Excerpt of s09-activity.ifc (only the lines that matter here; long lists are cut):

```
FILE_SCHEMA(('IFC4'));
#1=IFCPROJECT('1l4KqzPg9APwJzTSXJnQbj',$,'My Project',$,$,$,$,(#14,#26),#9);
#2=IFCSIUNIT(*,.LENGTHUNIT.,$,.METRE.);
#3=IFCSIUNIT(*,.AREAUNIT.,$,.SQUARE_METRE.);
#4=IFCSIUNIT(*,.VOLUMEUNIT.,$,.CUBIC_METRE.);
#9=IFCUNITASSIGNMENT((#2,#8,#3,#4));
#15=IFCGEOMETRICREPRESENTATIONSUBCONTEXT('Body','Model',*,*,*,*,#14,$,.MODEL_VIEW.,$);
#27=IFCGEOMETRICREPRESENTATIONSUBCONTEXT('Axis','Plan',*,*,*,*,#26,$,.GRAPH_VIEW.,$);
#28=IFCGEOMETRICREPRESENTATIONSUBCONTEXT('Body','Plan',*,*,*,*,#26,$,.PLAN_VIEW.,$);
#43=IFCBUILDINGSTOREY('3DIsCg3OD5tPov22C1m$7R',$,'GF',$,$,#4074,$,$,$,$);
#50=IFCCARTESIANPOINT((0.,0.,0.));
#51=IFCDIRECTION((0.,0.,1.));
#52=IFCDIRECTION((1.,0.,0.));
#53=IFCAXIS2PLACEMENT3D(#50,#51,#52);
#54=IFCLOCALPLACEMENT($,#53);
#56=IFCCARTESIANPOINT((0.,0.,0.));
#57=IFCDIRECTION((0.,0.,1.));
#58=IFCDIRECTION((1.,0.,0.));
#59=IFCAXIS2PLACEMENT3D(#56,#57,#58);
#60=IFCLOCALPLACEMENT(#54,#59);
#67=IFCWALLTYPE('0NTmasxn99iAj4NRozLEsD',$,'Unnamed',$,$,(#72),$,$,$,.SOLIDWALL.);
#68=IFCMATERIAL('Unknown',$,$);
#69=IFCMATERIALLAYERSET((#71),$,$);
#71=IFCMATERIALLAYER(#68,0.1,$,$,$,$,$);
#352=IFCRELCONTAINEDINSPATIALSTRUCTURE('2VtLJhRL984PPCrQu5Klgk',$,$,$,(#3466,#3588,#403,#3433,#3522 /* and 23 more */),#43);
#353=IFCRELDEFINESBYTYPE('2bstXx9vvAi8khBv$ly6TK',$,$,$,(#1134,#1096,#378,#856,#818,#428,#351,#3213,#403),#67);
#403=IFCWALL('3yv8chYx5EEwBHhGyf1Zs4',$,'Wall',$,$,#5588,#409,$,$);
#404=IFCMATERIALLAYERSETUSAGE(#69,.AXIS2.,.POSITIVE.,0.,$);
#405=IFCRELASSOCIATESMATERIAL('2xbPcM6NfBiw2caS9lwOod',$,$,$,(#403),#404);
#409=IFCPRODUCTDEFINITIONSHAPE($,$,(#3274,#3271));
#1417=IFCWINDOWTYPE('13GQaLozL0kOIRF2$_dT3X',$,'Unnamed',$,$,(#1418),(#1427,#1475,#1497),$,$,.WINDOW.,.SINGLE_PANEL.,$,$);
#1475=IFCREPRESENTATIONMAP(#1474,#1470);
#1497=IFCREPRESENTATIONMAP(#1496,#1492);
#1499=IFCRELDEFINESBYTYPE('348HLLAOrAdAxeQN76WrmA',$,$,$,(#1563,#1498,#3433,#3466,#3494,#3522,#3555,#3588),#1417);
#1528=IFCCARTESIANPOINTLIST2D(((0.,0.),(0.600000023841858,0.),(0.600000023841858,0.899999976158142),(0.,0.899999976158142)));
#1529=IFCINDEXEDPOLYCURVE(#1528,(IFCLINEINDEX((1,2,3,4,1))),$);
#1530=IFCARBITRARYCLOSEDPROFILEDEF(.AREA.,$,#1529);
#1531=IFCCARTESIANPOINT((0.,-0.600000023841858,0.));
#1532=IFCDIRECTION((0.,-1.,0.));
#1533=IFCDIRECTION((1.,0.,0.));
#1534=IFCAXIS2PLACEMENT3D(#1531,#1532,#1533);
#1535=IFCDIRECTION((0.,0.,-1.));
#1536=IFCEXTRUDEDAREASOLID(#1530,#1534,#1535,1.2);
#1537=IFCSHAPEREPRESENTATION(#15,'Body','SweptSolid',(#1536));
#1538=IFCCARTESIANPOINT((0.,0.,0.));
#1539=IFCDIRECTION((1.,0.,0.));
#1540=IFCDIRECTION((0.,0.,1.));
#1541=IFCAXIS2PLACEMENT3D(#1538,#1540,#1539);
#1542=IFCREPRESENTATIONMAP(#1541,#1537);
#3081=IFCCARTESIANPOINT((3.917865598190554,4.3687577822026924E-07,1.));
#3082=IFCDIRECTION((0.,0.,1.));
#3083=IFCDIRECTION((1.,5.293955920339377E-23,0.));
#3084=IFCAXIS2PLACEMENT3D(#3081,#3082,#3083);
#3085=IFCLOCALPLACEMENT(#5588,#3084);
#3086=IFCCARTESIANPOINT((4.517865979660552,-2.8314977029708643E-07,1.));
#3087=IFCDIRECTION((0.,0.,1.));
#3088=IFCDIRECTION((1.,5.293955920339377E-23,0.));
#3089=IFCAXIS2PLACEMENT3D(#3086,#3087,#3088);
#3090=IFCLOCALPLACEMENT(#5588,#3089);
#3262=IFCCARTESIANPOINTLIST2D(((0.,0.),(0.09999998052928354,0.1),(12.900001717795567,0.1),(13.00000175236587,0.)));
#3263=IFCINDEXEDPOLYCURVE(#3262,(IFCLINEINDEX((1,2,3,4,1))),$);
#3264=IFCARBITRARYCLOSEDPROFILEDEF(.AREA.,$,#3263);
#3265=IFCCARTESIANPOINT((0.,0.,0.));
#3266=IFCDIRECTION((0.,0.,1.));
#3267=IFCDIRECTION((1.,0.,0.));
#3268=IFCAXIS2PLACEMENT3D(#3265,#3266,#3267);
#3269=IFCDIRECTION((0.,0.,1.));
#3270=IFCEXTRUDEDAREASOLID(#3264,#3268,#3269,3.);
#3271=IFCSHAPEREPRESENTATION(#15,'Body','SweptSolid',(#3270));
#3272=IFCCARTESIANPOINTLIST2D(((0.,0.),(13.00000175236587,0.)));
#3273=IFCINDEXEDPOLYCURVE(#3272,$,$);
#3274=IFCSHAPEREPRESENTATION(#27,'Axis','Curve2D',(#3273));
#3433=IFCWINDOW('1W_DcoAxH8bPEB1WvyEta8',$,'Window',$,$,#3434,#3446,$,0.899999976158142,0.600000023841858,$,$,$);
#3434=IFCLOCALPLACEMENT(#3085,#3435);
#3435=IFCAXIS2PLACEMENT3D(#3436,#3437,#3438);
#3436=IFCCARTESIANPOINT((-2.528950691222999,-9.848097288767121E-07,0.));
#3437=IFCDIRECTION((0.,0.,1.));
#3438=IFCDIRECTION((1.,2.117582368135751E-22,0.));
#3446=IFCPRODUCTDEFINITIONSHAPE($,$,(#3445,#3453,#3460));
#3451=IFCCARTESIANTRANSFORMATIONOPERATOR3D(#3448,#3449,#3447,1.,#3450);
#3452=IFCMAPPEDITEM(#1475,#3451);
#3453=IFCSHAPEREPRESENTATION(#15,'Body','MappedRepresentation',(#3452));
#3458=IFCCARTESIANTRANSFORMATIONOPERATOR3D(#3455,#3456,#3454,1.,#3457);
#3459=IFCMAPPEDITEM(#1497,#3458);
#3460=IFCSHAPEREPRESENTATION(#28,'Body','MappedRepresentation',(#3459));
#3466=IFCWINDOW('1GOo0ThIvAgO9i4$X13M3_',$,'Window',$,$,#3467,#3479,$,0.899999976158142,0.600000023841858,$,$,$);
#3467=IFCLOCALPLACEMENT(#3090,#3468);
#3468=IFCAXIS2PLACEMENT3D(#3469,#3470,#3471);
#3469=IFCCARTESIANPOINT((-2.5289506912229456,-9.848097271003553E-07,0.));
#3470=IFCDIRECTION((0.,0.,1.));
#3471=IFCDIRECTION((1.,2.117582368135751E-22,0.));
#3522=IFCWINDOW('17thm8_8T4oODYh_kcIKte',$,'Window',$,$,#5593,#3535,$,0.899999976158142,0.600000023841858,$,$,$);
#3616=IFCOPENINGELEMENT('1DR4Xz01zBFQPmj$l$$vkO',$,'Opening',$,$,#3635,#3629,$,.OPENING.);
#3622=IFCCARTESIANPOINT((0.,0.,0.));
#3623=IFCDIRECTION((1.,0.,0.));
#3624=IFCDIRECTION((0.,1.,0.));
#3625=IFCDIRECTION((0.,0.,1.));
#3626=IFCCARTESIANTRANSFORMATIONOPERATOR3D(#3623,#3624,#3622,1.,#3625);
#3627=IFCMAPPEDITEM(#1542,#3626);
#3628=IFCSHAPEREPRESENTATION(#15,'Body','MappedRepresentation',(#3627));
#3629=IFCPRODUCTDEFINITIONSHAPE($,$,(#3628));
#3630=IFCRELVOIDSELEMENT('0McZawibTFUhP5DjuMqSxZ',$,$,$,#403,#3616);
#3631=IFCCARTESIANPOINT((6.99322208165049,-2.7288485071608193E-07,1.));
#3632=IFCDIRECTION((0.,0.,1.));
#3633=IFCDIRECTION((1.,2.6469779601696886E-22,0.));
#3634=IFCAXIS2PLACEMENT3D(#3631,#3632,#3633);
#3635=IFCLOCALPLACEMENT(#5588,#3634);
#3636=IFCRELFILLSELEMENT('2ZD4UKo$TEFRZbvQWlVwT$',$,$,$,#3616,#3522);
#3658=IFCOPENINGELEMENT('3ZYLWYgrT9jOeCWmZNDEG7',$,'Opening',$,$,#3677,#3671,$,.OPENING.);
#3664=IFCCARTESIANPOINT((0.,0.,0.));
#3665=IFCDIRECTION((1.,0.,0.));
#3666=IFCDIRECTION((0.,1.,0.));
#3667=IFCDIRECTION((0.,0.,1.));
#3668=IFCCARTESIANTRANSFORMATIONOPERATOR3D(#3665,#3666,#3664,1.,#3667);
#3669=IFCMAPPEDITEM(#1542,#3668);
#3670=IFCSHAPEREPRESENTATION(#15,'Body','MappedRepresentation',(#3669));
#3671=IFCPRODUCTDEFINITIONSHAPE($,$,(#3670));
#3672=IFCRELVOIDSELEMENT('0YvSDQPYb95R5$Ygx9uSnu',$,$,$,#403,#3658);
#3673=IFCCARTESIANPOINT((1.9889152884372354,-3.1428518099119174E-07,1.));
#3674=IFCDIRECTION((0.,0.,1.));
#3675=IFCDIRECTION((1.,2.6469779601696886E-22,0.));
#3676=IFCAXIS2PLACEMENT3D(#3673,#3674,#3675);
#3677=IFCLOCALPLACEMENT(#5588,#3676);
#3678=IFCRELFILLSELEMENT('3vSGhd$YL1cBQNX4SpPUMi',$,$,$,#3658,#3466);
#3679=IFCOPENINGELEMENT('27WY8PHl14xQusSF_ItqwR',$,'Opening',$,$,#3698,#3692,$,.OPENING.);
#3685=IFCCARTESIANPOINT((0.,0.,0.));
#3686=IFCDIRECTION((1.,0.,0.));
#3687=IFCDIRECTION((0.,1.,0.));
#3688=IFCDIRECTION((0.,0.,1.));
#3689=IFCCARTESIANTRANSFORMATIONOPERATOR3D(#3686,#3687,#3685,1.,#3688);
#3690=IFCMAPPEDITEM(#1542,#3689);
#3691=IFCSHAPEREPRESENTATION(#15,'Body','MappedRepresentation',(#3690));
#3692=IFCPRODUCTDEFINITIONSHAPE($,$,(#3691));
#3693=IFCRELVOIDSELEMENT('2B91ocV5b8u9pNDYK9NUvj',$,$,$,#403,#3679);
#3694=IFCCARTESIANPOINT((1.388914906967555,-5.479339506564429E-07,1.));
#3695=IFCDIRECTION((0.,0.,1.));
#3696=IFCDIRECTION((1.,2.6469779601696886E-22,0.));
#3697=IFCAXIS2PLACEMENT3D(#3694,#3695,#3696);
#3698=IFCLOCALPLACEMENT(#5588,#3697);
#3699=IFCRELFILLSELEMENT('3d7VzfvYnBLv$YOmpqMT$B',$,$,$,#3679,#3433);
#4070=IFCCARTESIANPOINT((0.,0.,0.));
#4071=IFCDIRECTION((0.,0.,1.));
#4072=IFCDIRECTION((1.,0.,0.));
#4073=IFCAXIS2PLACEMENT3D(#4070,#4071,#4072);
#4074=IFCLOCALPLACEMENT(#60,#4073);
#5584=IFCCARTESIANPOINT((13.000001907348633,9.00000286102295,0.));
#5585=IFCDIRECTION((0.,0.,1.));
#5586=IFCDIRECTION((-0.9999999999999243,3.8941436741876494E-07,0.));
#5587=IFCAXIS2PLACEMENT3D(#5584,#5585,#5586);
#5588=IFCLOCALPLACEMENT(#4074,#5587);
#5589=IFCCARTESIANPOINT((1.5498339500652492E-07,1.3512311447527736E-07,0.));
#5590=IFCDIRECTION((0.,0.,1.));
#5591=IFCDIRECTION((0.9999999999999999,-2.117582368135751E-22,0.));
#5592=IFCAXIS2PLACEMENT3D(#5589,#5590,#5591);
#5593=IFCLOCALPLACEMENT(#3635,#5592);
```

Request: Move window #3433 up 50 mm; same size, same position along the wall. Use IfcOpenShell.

```python
import numpy as np
import ifcopenshell
import ifcopenshell.api.geometry
import ifcopenshell.util.placement
import ifcopenshell.util.unit

model = ifcopenshell.open("s09-activity.ifc")
unit_scale = ifcopenshell.util.unit.calculate_unit_scale(model)

window = model.by_guid("1W_DcoAxH8bPEB1WvyEta8")
opening = window.FillsVoids[0].RelatingOpeningElement
dz = 0.05 / unit_scale

shift = np.array([0.0, 0.0, dz])
# The window is not placed relative to its opening, so move both.
for product in (opening, window):
    matrix = ifcopenshell.util.placement.get_local_placement(product.ObjectPlacement)
    matrix[:3, 3] += shift
    ifcopenshell.api.geometry.edit_object_placement(model, product=product, matrix=matrix, is_si=False)

print(f"moved by {dz * unit_scale:+.3f} m")

model.write("s09-activity_edited.ifc")
```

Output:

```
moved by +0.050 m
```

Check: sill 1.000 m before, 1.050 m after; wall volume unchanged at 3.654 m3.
